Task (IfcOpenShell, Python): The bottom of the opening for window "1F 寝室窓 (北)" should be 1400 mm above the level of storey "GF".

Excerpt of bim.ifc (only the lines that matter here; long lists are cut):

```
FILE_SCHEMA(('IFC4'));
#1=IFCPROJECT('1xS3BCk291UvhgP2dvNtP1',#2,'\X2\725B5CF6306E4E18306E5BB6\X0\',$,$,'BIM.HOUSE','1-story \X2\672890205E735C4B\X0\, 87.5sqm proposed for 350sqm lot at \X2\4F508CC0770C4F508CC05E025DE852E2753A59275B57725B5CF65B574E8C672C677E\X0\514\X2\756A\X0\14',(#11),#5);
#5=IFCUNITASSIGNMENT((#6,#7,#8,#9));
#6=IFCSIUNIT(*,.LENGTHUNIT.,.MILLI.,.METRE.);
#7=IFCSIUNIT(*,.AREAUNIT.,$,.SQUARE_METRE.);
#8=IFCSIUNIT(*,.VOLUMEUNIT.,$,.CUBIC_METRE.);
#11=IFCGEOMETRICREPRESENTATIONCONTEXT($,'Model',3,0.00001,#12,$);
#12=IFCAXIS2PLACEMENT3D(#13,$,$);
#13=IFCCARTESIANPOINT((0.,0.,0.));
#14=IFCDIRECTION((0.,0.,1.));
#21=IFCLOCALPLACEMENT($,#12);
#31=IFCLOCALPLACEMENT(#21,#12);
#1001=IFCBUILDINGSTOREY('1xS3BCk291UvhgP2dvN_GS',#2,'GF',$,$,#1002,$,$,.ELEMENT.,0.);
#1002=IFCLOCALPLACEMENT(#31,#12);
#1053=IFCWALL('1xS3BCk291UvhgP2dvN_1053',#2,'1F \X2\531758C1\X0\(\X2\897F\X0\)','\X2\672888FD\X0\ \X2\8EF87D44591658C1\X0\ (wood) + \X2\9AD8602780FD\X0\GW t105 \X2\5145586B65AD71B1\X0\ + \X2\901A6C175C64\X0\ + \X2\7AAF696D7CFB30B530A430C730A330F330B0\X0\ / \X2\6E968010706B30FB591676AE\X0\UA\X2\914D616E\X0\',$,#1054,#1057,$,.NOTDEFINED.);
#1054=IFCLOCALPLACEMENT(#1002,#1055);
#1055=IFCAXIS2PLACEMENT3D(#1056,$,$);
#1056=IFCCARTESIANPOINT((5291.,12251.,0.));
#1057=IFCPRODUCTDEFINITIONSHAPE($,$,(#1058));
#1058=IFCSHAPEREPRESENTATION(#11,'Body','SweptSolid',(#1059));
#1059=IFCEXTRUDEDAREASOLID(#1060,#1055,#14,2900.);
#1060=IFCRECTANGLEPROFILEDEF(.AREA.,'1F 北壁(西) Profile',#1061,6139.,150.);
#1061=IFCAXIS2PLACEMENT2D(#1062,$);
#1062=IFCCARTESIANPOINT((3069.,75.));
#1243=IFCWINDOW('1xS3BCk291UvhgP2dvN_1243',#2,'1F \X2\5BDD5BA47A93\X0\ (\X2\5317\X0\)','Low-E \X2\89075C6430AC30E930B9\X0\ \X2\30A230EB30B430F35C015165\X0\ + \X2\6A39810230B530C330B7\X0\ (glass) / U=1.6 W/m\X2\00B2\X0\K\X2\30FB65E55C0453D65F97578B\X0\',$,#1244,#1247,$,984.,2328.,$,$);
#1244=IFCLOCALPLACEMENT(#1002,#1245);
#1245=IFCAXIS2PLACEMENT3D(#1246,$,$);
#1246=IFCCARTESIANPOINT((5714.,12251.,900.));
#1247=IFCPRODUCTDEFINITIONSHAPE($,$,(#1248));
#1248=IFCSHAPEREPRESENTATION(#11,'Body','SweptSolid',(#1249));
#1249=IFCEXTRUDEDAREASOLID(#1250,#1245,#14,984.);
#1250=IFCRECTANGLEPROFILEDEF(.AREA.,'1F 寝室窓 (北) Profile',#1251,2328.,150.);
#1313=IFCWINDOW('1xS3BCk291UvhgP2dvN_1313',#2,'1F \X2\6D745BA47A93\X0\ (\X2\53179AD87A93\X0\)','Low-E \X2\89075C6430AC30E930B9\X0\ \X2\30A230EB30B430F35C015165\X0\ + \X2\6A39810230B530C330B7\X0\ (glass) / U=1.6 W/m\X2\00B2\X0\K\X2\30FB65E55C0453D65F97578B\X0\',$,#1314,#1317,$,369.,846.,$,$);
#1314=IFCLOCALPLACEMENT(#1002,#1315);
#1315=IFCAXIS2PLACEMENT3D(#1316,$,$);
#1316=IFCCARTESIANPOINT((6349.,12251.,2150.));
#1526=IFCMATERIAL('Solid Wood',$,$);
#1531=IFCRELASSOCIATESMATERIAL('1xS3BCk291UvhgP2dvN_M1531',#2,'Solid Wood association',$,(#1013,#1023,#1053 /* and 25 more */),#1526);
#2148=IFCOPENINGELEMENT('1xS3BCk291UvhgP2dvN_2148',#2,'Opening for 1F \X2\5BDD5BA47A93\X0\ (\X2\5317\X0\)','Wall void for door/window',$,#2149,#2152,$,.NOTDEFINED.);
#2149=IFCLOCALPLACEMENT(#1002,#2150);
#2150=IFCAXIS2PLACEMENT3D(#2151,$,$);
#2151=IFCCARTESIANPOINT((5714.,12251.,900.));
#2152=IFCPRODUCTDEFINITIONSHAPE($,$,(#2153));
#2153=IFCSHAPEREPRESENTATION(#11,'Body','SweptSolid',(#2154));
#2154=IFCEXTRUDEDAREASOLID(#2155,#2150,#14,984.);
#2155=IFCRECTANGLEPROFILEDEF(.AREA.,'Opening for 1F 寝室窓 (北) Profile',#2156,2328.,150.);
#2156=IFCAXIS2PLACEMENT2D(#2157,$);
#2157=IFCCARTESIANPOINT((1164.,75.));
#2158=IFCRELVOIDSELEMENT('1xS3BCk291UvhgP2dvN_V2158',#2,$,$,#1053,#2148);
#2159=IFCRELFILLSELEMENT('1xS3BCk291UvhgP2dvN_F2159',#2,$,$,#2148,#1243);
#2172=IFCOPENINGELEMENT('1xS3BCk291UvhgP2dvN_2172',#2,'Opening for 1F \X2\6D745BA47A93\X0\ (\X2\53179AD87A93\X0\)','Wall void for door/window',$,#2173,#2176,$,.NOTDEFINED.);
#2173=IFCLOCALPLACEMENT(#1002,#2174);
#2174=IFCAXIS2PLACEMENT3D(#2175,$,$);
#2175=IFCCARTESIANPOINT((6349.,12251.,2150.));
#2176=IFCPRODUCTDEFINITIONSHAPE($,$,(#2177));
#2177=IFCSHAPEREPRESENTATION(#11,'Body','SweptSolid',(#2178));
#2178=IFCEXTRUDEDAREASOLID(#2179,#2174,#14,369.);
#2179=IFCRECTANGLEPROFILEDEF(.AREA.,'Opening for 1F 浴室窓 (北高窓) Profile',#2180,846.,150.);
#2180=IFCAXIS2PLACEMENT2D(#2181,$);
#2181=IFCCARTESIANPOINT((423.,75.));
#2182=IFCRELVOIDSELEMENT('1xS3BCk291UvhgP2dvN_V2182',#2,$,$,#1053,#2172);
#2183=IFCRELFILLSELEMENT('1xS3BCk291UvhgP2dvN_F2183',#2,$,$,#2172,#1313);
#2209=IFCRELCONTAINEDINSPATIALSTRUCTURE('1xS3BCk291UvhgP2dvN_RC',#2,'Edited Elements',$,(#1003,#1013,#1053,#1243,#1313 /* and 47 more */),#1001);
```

```python
import numpy as np
import ifcopenshell
import ifcopenshell.api.geometry
import ifcopenshell.geom
import ifcopenshell.util.element
import ifcopenshell.util.placement
import ifcopenshell.util.shape
import ifcopenshell.util.unit

model = ifcopenshell.open("bim.ifc")
unit_scale = ifcopenshell.util.unit.calculate_unit_scale(model)

window = model.by_guid("1xS3BCk291UvhgP2dvN_1243")
opening = window.FillsVoids[0].RelatingOpeningElement
storey = ifcopenshell.util.element.get_container(window, ifc_class="IfcBuildingStorey")
level = ifcopenshell.util.placement.get_local_placement(storey.ObjectPlacement)[2, 3]

# The opening's origin need not be at the sill, so measure its lowest point.
shape = ifcopenshell.geom.create_shape(ifcopenshell.geom.settings(), opening)
bottom = ifcopenshell.util.shape.get_shape_bottom_elevation(shape, shape.geometry) / unit_scale
dz = level + 1.4 / unit_scale - bottom

shift = np.array([0.0, 0.0, dz])
# The window is not placed relative to its opening, so move both.
for product in (opening, window):
    matrix = ifcopenshell.util.placement.get_local_placement(product.ObjectPlacement)
    matrix[:3, 3] += shift
    ifcopenshell.api.geometry.edit_object_placement(model, product=product, matrix=matrix, is_si=False)

print(f"moved by {dz * unit_scale:+.3f} m")

model.write("bim_edited.ifc")
```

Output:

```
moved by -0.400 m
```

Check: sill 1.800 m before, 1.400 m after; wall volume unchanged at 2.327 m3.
